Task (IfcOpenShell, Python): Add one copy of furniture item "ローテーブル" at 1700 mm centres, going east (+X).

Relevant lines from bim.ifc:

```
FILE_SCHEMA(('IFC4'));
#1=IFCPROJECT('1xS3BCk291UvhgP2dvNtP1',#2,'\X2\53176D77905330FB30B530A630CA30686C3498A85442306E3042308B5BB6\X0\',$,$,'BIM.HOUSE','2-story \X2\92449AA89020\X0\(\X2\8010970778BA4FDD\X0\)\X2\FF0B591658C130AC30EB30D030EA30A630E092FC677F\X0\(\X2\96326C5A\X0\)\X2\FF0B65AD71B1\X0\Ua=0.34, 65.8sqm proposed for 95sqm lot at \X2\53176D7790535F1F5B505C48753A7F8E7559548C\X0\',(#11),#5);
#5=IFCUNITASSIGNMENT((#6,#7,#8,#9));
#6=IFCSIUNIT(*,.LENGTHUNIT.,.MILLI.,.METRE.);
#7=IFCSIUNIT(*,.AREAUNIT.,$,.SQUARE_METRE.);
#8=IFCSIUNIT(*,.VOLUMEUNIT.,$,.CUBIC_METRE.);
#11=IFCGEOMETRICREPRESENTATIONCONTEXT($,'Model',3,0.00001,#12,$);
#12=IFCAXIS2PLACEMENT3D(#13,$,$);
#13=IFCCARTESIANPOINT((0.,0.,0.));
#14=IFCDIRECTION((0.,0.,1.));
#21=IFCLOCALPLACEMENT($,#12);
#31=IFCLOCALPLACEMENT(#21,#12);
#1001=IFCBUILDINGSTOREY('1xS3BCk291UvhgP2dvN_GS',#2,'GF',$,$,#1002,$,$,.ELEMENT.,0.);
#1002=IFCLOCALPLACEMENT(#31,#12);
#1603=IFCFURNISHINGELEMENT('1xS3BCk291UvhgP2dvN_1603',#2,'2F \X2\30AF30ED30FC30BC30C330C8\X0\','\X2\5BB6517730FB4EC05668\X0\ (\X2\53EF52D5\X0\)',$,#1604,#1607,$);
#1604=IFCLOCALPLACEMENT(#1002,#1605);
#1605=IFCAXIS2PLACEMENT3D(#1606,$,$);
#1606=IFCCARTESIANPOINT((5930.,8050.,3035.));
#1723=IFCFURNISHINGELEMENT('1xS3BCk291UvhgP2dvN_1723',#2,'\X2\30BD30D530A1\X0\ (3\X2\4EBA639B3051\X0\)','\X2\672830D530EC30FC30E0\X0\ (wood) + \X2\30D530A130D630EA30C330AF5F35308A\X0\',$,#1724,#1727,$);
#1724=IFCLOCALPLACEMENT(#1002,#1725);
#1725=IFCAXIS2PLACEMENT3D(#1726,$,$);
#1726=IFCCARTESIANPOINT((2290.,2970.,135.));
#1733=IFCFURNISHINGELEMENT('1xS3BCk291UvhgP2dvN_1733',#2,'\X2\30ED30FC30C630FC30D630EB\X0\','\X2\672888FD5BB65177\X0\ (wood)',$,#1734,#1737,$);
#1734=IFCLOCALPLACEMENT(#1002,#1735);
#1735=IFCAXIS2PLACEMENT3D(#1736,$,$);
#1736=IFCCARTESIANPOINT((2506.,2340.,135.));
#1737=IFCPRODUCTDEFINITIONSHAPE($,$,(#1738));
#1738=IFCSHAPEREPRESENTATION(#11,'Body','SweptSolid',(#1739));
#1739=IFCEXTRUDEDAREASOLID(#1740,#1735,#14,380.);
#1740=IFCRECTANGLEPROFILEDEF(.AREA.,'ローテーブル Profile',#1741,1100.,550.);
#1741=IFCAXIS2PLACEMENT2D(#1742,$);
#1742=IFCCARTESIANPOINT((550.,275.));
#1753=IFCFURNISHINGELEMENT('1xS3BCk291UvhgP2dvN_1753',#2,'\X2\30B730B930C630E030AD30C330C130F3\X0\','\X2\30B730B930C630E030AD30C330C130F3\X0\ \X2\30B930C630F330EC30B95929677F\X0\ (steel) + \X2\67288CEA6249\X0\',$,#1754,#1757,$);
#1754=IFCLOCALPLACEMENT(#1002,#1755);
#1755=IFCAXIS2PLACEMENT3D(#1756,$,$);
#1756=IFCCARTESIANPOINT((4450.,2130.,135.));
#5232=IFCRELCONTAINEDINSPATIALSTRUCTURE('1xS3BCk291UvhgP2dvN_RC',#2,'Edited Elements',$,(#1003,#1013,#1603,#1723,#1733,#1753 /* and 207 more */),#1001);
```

```python
import numpy as np
import ifcopenshell
import ifcopenshell.api.geometry
import ifcopenshell.api.root
import ifcopenshell.util.element
import ifcopenshell.util.placement

model = ifcopenshell.open("bim.ifc")


def reuse_history(source, copy):
    """copy_class also copies each property set's owner history, people and application; keep the originals."""
    for rel in copy.IsDefinedBy:
        if rel.is_a("IfcRelDefinesByProperties") and (history := rel.RelatingPropertyDefinition.OwnerHistory):
            rel.RelatingPropertyDefinition.OwnerHistory = source.OwnerHistory
            ifcopenshell.util.element.remove_deep2(model, history)


source = model.by_id(1733)
base = ifcopenshell.util.placement.get_local_placement(source.ObjectPlacement)
step = np.array([1.0, 0.0, 0.0]) * 1700.0

for i in range(1, 2):
    copy = ifcopenshell.api.root.copy_class(model, product=source)
    copy.Representation = ifcopenshell.util.element.copy_deep(
        model, source.Representation, exclude=["IfcGeometricRepresentationContext", "IfcRepresentationMap"]
    )
    reuse_history(source, copy)
    matrix = base.copy()
    matrix[:3, 3] += i * step
    print("added at", matrix[:3, 3].round(3) + 0.0)
    ifcopenshell.api.geometry.edit_object_placement(model, product=copy, matrix=matrix, is_si=False)

model.write("bim_rev.ifc")
```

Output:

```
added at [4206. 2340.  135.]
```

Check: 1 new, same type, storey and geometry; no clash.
